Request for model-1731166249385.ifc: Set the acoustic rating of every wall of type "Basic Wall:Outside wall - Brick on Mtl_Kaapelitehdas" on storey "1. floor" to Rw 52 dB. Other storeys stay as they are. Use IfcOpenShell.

First a look at what the model holds.

```python
import ifcopenshell
import ifcopenshell.util.element

model = ifcopenshell.open("model-1731166249385.ifc")
print(model.schema)
storey = next(s for s in model.by_type("IfcBuildingStorey") if s.Name == "1. floor")
walls = [e for e in ifcopenshell.util.element.get_decomposition(storey) if e.is_a("IfcWall")]
seen = {}
for e in walls:
    element_type = ifcopenshell.util.element.get_type(e)
    key = (element_type.Name if element_type != e and element_type else None, ifcopenshell.util.element.get_pset(e, "Pset_WallCommon", "AcousticRating"))
    seen[key] = seen.get(key, 0) + 1
for (name, value), count in sorted(seen.items(), key=str):
    print(count, "x", name, "|", value)
```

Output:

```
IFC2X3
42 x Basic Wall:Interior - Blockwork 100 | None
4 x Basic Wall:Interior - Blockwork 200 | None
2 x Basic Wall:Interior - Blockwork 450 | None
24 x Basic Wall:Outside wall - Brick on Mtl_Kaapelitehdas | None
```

```python
import ifcopenshell
import ifcopenshell.api.pset
import ifcopenshell.util.element

model = ifcopenshell.open("model-1731166249385.ifc")

storey = next(s for s in model.by_type("IfcBuildingStorey") if s.Name == "1. floor")
walls = [e for e in ifcopenshell.util.element.get_decomposition(storey) if e.is_a("IfcWall")]

count = 0
for e in walls:
    element_type = ifcopenshell.util.element.get_type(e)
    if element_type in (None, e) or element_type.Name != "Basic Wall:Outside wall - Brick on Mtl_Kaapelitehdas":
        continue
    # add_pset returns the element's existing set when there is one.
    pset = ifcopenshell.api.pset.add_pset(model, product=e, name="Pset_WallCommon")
    ifcopenshell.api.pset.edit_pset(model, pset=pset, properties={"AcousticRating": "Rw 52 dB"})
    count += 1

print(count, "walls updated")

model.write("model-1731166249385_updated.ifc")
```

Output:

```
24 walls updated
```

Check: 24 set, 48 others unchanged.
